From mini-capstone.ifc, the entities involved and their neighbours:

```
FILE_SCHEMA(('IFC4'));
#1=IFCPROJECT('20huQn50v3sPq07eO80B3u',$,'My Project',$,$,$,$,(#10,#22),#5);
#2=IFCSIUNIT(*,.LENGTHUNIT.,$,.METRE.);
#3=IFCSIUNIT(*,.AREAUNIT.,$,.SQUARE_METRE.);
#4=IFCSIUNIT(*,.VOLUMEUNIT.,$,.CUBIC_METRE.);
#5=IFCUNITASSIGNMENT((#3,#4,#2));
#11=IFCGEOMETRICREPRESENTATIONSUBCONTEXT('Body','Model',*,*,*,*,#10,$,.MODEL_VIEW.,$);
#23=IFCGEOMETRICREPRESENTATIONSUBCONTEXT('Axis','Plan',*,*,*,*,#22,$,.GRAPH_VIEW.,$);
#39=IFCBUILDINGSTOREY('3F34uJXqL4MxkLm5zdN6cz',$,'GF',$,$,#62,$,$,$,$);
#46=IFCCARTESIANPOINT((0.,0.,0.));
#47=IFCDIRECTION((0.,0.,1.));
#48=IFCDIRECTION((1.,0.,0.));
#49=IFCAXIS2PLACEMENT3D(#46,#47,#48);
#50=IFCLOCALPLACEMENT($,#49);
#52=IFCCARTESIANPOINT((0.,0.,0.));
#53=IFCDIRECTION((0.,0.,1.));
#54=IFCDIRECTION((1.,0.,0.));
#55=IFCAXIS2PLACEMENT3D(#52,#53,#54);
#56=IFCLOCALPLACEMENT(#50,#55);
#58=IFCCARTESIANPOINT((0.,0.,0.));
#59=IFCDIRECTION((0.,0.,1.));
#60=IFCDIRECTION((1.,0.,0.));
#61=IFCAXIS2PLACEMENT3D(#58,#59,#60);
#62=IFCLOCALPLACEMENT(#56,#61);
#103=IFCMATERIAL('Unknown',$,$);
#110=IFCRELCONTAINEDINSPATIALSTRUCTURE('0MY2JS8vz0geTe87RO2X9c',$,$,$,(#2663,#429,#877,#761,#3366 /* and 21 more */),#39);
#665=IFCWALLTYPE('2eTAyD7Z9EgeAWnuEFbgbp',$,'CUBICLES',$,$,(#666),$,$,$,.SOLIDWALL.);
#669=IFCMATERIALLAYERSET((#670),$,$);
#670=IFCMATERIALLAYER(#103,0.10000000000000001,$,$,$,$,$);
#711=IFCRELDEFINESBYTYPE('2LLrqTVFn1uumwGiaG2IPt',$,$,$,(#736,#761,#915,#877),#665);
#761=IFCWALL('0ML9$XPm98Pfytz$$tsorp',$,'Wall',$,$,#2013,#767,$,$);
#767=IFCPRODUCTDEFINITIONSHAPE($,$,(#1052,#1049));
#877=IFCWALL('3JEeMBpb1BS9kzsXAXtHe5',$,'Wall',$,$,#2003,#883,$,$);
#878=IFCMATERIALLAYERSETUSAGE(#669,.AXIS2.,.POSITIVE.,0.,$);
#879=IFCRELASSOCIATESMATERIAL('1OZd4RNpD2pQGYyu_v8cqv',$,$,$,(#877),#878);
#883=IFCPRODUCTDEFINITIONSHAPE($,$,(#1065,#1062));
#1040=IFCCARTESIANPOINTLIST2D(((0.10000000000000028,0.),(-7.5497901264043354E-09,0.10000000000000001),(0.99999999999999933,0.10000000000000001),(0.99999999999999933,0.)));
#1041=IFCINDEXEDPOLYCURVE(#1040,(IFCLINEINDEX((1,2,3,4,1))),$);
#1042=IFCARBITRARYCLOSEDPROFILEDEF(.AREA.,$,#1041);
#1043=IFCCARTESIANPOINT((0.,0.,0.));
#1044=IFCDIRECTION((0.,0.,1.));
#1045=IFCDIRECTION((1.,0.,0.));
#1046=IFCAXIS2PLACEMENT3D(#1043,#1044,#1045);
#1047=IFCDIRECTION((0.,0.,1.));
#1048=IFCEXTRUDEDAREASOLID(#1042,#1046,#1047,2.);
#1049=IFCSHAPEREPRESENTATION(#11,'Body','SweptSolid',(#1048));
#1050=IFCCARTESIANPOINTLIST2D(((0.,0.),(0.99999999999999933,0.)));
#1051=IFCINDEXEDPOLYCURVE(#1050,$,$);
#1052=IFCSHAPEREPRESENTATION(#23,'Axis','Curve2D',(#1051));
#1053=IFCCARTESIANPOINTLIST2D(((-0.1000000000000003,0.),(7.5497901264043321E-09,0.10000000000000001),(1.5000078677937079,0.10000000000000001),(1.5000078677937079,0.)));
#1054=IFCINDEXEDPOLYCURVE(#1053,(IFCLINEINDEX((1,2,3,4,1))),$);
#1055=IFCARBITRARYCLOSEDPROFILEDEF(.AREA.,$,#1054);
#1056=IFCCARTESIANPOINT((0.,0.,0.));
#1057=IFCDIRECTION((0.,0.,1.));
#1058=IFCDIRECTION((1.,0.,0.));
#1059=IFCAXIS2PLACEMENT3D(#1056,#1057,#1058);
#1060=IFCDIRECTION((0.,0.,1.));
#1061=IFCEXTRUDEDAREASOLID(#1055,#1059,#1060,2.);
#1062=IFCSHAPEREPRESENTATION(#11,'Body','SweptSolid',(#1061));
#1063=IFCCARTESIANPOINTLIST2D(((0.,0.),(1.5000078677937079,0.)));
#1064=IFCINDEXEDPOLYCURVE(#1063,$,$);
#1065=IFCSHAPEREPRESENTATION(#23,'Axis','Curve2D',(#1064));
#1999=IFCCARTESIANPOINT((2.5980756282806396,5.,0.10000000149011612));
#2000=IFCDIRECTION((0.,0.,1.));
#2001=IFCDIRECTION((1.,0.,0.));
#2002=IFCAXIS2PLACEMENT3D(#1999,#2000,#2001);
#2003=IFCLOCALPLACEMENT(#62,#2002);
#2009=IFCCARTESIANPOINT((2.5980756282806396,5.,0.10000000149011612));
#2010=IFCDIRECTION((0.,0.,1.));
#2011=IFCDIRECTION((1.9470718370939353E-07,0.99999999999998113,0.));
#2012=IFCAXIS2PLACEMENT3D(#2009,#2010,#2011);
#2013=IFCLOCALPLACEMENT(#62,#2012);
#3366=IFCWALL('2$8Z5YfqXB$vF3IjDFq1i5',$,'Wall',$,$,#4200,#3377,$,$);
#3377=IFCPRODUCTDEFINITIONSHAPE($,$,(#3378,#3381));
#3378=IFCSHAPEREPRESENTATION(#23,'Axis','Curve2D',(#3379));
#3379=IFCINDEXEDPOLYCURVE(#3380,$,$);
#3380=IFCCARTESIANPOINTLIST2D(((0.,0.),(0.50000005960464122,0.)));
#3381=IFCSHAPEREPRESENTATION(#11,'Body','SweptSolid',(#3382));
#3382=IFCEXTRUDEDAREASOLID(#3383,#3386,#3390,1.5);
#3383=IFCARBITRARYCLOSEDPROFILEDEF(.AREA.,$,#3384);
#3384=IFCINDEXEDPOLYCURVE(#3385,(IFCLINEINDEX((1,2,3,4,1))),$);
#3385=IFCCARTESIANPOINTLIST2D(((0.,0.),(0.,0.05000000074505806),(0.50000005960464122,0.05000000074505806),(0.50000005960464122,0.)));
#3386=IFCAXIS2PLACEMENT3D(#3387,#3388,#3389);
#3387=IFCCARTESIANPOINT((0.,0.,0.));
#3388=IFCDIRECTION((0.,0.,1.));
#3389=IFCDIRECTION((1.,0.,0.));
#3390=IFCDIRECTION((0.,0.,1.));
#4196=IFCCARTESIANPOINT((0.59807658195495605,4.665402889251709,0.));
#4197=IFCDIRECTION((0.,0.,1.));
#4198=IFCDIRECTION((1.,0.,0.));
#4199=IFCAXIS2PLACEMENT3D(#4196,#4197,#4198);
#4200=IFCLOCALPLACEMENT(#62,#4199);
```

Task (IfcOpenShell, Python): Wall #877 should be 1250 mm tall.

```python
import ifcopenshell
import ifcopenshell.geom
import ifcopenshell.util.representation
import ifcopenshell.util.shape
import ifcopenshell.util.unit

model = ifcopenshell.open("mini-capstone.ifc")
unit_scale = ifcopenshell.util.unit.calculate_unit_scale(model)
settings = ifcopenshell.geom.settings()


def volume(element):
    """Net volume in cubic metres, openings subtracted."""
    shape = ifcopenshell.geom.create_shape(settings, element)
    return ifcopenshell.util.shape.get_volume(shape.geometry)


wall = model.by_guid("3JEeMBpb1BS9kzsXAXtHe5")
before = volume(wall)

body = ifcopenshell.util.representation.get_representation(wall, "Model", "Body")
solid = body.Items[0]
old_height = solid.Depth
solid.Depth = 1.25 / unit_scale
after = volume(wall)

print(f"height {old_height:g} -> {solid.Depth:g}, volume {before:.3f} -> {after:.3f} m3")

model.write("mini-capstone_rev.ifc")
```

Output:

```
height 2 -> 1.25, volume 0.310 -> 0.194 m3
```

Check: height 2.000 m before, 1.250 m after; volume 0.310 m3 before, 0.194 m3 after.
